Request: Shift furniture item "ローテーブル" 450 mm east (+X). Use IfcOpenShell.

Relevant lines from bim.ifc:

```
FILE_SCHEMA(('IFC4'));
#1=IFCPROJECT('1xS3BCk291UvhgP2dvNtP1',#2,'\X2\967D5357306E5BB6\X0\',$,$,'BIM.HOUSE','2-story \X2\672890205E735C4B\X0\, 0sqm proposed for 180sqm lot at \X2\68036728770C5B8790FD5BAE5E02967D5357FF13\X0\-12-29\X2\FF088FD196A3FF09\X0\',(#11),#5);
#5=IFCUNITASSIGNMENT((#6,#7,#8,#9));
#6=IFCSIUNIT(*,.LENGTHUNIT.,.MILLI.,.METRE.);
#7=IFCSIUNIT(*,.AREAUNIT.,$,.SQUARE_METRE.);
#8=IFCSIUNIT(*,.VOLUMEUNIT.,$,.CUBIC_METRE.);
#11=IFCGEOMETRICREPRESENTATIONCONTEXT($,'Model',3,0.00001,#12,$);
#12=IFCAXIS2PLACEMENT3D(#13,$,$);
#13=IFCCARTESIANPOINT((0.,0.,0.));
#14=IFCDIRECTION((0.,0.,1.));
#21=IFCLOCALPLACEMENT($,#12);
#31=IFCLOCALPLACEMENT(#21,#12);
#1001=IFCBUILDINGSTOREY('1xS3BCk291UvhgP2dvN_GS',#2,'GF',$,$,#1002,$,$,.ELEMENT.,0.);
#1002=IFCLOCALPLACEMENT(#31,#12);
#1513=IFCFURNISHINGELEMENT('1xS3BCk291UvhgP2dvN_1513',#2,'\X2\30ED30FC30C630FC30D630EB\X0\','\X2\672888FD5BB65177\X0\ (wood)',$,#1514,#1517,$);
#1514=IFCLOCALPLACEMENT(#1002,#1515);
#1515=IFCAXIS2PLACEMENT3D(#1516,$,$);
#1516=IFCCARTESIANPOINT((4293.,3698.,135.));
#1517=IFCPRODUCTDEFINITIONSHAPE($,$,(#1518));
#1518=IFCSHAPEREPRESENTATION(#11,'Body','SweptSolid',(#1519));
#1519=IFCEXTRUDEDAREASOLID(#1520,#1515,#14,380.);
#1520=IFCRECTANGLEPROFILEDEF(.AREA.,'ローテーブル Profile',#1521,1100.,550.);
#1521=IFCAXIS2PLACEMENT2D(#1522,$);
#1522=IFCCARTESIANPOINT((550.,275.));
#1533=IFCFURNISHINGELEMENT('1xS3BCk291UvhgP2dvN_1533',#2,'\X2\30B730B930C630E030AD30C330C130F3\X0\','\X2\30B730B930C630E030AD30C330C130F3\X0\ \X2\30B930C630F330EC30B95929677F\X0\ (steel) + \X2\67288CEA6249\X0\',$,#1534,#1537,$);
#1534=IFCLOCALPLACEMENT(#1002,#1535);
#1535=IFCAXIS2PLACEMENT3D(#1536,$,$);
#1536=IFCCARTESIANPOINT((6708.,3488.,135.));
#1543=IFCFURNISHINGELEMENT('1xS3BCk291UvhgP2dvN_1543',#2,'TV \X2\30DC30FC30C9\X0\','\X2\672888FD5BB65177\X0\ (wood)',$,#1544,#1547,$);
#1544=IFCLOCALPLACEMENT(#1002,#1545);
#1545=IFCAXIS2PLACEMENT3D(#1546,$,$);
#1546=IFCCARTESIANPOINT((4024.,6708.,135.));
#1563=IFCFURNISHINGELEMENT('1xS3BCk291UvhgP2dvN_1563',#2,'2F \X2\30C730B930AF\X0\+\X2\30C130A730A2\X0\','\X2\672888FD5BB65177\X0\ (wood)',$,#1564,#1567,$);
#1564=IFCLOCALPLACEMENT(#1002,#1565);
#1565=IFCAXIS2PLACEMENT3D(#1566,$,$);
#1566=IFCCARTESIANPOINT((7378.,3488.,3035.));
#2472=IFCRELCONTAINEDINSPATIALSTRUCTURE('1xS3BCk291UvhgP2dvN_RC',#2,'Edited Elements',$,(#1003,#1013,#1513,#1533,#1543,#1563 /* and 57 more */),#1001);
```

```python
import ifcopenshell
import ifcopenshell.api.geometry
import ifcopenshell.util.placement

model = ifcopenshell.open("bim.ifc")

item = model.by_guid("1xS3BCk291UvhgP2dvN_1513")
matrix = ifcopenshell.util.placement.get_local_placement(item.ObjectPlacement)
matrix[0, 3] += 450.0
ifcopenshell.api.geometry.edit_object_placement(model, product=item, matrix=matrix, is_si=False)

print(ifcopenshell.util.placement.get_local_placement(item.ObjectPlacement).round(3) + 0.0)

model.write("bim_v2.ifc")
```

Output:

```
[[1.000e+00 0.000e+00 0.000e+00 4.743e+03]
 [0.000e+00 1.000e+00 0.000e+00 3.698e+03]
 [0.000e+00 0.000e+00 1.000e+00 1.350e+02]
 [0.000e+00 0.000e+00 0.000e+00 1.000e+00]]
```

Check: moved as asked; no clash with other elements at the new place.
